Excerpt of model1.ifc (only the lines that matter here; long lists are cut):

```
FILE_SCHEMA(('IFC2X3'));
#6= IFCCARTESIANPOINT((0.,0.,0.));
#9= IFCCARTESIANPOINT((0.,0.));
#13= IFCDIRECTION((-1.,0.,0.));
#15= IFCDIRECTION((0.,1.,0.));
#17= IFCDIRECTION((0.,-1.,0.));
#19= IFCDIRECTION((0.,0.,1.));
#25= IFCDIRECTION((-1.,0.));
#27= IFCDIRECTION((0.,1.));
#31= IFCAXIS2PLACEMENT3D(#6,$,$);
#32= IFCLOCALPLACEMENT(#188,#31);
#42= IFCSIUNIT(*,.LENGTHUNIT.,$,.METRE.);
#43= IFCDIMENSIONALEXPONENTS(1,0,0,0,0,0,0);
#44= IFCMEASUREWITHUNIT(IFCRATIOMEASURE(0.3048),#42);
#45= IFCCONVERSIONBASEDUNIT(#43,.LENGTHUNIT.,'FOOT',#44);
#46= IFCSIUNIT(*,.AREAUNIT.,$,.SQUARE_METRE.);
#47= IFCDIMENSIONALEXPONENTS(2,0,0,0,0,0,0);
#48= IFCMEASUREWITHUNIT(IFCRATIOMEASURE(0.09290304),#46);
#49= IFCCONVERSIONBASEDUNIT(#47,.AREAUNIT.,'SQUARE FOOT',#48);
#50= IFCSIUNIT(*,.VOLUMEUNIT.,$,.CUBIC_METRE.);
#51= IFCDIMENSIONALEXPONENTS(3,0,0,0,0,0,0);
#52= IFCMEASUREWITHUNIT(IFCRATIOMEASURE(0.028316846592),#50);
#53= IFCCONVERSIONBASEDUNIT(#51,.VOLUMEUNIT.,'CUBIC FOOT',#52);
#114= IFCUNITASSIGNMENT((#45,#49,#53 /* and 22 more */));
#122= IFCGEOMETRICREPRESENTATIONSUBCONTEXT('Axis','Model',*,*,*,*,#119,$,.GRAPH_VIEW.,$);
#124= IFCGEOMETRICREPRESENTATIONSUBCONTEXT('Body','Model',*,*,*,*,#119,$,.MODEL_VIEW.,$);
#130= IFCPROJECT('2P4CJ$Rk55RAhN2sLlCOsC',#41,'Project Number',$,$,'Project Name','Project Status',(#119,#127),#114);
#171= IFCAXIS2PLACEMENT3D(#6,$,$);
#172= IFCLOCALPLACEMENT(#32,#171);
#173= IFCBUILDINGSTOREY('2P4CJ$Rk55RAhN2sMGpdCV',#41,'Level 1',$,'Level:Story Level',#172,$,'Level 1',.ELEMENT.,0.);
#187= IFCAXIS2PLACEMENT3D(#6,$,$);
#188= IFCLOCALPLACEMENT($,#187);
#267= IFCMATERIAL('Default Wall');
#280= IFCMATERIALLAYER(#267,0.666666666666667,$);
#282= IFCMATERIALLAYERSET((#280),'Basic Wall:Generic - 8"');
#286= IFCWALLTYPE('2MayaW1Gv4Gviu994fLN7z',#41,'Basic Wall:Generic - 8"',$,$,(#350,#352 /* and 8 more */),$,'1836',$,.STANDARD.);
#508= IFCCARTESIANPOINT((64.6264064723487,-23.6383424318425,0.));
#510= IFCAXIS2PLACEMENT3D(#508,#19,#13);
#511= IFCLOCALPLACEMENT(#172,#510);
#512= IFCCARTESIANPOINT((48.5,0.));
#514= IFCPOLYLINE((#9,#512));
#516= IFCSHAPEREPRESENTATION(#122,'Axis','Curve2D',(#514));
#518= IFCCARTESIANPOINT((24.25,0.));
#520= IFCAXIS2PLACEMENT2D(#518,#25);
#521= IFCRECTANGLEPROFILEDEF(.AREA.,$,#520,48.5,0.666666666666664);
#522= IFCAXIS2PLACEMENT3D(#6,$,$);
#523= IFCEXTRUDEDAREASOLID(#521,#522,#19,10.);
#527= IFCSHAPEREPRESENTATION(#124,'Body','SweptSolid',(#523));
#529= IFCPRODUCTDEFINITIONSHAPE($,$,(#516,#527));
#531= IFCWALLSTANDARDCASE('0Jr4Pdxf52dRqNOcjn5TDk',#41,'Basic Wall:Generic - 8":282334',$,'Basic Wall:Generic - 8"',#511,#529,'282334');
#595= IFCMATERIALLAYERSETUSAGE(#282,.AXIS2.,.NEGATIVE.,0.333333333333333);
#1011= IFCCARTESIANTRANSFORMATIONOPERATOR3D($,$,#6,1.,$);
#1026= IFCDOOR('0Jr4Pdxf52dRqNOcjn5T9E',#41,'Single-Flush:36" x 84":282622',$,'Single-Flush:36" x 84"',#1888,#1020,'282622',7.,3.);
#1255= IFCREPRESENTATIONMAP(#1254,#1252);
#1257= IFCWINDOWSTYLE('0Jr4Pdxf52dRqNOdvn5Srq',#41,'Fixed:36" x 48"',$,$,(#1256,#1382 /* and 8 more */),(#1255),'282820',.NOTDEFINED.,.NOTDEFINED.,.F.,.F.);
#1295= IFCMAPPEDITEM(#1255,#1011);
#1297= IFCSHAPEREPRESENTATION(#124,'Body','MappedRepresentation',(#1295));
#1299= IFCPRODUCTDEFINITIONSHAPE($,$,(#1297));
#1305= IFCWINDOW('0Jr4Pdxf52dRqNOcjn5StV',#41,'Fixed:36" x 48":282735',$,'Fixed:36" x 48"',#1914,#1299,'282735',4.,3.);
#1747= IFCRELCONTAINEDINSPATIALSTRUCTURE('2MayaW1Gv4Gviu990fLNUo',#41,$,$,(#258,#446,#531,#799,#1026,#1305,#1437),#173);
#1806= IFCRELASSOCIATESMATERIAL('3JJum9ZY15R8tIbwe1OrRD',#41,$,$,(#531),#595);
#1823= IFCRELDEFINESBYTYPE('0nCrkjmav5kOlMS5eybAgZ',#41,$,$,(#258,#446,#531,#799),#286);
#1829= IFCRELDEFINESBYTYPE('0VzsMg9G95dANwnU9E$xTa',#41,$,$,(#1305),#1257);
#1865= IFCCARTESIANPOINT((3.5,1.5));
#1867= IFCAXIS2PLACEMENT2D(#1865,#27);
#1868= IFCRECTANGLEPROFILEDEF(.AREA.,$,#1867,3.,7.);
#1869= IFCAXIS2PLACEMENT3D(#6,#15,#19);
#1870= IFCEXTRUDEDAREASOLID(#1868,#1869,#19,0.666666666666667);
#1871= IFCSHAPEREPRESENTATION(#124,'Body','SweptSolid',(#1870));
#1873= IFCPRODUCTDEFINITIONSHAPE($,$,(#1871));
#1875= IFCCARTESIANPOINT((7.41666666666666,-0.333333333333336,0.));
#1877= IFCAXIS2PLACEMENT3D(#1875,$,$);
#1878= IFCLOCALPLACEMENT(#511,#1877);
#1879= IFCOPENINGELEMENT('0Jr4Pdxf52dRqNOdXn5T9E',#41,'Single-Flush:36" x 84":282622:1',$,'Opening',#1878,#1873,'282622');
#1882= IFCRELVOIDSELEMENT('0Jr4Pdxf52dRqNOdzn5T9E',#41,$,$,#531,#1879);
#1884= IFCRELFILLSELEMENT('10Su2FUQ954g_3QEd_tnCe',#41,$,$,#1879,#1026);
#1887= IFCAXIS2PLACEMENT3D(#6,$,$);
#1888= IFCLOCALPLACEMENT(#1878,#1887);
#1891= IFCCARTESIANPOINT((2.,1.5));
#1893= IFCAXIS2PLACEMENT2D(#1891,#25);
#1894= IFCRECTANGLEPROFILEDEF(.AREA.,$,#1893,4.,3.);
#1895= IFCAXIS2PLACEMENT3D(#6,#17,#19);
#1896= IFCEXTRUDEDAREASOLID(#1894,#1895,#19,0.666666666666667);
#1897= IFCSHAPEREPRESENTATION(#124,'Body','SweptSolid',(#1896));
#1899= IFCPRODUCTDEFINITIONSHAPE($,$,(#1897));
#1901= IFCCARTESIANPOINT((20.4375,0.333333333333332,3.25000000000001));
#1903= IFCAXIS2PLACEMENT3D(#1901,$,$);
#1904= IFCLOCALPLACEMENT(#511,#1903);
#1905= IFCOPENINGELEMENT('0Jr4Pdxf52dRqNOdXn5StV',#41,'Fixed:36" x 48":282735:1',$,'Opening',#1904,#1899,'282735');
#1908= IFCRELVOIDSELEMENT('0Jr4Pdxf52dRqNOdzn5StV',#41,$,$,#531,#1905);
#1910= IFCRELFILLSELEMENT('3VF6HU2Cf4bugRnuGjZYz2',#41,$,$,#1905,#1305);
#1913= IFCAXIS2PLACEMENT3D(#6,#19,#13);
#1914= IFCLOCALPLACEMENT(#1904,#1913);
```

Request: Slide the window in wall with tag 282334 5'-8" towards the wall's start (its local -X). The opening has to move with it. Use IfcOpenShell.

```python
import ifcopenshell
import ifcopenshell.api.geometry
import ifcopenshell.util.placement
import ifcopenshell.util.unit

model = ifcopenshell.open("model1.ifc")
unit_scale = ifcopenshell.util.unit.calculate_unit_scale(model)

window = model.by_guid("0Jr4Pdxf52dRqNOcjn5StV")
opening = window.FillsVoids[0].RelatingOpeningElement
wall = opening.VoidsElements[0].RelatingBuildingElement

wall_matrix = ifcopenshell.util.placement.get_local_placement(wall.ObjectPlacement)
shift = wall_matrix[:3, 0] * -68 * 0.0254 / unit_scale
before = ifcopenshell.util.placement.get_local_placement(window.ObjectPlacement)[:3, 3].copy()

# The window is placed relative to its opening, so it follows when the opening moves.
matrix = ifcopenshell.util.placement.get_local_placement(opening.ObjectPlacement)
matrix[:3, 3] += shift
ifcopenshell.api.geometry.edit_object_placement(
    model, product=opening, matrix=matrix, is_si=False, should_transform_children=True
)

after = ifcopenshell.util.placement.get_local_placement(window.ObjectPlacement)[:3, 3]
print("window moved by", (after - before).round(3) + 0.0)

model.write("model1_updated.ifc")
```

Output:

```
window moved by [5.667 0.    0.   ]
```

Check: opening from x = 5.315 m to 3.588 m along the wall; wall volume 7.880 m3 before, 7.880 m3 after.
